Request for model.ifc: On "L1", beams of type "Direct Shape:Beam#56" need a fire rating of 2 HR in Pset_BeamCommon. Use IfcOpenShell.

First a look at what the model holds.

```python
import ifcopenshell
import ifcopenshell.util.element

model = ifcopenshell.open("model.ifc")
print(model.schema)
storey = next(s for s in model.by_type("IfcBuildingStorey") if s.Name == "L1")
beams = [e for e in ifcopenshell.util.element.get_decomposition(storey) if e.is_a("IfcBeam")]
seen = {}
for e in beams:
    element_type = ifcopenshell.util.element.get_type(e)
    key = (element_type.Name if element_type != e and element_type else None, ifcopenshell.util.element.get_pset(e, "Pset_BeamCommon", "FireRating"))
    seen[key] = seen.get(key, 0) + 1
for (name, value), count in sorted(seen.items(), key=str):
    print(count, "x", name, "|", value)
```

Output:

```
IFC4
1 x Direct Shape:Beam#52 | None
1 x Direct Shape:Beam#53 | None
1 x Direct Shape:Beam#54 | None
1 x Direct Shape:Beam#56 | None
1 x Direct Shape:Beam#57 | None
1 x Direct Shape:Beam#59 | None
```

```python
import ifcopenshell
import ifcopenshell.api.pset
import ifcopenshell.util.element

model = ifcopenshell.open("model.ifc")

storey = next(s for s in model.by_type("IfcBuildingStorey") if s.Name == "L1")
beams = [e for e in ifcopenshell.util.element.get_decomposition(storey) if e.is_a("IfcBeam")]

count = 0
for e in beams:
    element_type = ifcopenshell.util.element.get_type(e)
    if element_type in (None, e) or element_type.Name != "Direct Shape:Beam#56":
        continue
    # add_pset returns the element's existing set when there is one.
    pset = ifcopenshell.api.pset.add_pset(model, product=e, name="Pset_BeamCommon")
    ifcopenshell.api.pset.edit_pset(model, pset=pset, properties={"FireRating": "2 HR"})
    count += 1

print(count, "beams updated")

model.write("model_edited.ifc")
```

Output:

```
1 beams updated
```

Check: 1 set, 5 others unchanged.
